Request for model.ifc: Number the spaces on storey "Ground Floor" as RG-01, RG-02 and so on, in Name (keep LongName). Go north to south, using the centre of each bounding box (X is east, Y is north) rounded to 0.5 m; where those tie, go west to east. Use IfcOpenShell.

First a look at what the model holds.

```python
import ifcopenshell
import ifcopenshell.util.element
import ifcopenshell.util.placement

model = ifcopenshell.open("model.ifc")
print(model.schema)
storey = next(s for s in model.by_type("IfcBuildingStorey") if s.Name == "Ground Floor")
spaces = [e for e in ifcopenshell.util.element.get_decomposition(storey) if e.is_a("IfcSpace")]
for e in sorted(spaces, key=lambda e: e.id()):
    origin = ifcopenshell.util.placement.get_local_placement(e.ObjectPlacement)[:3, 3]
    print(e.id(), e.Name, e.LongName, origin.round(2) + 0.0, sep=" | ")
```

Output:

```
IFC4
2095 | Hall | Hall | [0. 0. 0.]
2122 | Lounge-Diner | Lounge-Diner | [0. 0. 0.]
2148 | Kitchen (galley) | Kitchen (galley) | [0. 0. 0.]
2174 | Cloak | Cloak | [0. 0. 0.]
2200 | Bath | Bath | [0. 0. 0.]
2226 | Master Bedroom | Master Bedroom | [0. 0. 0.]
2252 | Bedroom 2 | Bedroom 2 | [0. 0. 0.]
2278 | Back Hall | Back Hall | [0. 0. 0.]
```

```python
import ifcopenshell
import ifcopenshell.geom
import ifcopenshell.util.element
import ifcopenshell.util.shape

model = ifcopenshell.open("model.ifc")
settings = ifcopenshell.geom.settings()
settings.set("use-world-coords", True)


def centre(element):
    shape = ifcopenshell.geom.create_shape(settings, element)
    return ifcopenshell.util.shape.get_bbox_centroid(shape.geometry)


storey = next(s for s in model.by_type("IfcBuildingStorey") if s.Name == "Ground Floor")
spaces = [e for e in ifcopenshell.util.element.get_decomposition(storey) if e.is_a("IfcSpace")]

# Insertion points can sit at a corner or the storey origin, so sort by the geometry (in metres).
centres = {e: centre(e) for e in spaces}
spaces.sort(key=lambda e: (-round(centres[e][1] / 0.5), centres[e][0]))

for i, e in enumerate(spaces, start=1):
    number = f"RG-{i:02d}"
    e.Name = number
    print(e.id(), number)

model.write("model_v2.ifc")
```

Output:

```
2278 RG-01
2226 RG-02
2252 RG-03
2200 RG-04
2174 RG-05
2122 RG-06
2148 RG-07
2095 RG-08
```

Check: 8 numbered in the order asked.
